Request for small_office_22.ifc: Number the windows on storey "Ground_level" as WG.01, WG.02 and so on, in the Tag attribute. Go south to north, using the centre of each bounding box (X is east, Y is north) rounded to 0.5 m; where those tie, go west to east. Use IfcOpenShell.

First a look at what the model holds.

```python
import ifcopenshell
import ifcopenshell.util.element
import ifcopenshell.util.placement

model = ifcopenshell.open("small_office_22.ifc")
print(model.schema)
storey = next(s for s in model.by_type("IfcBuildingStorey") if s.Name == "Ground_level")
windows = [e for e in ifcopenshell.util.element.get_decomposition(storey) if e.is_a("IfcWindow")]
for e in sorted(windows, key=lambda e: e.id()):
    origin = ifcopenshell.util.placement.get_local_placement(e.ObjectPlacement)[:3, 3]
    print(e.id(), e.Tag, e.Name, origin.round(2) + 0.0, sep=" | ")
```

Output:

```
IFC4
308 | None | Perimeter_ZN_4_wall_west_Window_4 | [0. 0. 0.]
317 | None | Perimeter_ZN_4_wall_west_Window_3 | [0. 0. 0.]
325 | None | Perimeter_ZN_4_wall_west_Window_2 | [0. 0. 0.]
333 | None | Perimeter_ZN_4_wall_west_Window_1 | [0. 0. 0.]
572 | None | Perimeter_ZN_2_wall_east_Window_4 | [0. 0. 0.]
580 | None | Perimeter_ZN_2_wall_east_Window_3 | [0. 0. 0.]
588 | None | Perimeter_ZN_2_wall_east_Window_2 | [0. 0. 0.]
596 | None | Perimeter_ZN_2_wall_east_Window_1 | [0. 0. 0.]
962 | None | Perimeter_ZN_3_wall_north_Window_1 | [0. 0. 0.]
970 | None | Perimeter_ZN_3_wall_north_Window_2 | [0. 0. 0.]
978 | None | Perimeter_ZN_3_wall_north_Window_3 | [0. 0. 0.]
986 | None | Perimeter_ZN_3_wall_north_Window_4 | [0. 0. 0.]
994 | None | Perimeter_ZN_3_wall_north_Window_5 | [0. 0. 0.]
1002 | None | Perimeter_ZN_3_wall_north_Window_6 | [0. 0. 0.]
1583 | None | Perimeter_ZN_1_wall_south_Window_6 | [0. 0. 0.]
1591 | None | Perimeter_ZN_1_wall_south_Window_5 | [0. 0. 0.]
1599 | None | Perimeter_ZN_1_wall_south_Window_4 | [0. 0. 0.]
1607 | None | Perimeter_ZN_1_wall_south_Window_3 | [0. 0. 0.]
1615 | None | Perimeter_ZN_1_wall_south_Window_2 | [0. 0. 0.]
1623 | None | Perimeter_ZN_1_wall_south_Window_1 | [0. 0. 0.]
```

```python
import ifcopenshell
import ifcopenshell.geom
import ifcopenshell.util.element
import ifcopenshell.util.shape

model = ifcopenshell.open("small_office_22.ifc")
settings = ifcopenshell.geom.settings()
settings.set("use-world-coords", True)


def centre(element):
    shape = ifcopenshell.geom.create_shape(settings, element)
    return ifcopenshell.util.shape.get_bbox_centroid(shape.geometry)


storey = next(s for s in model.by_type("IfcBuildingStorey") if s.Name == "Ground_level")
windows = [e for e in ifcopenshell.util.element.get_decomposition(storey) if e.is_a("IfcWindow")]

# Insertion points can sit at a corner or the storey origin, so sort by the geometry (in metres).
centres = {e: centre(e) for e in windows}
windows.sort(key=lambda e: (round(centres[e][1] / 0.5), centres[e][0]))

for i, e in enumerate(windows, start=1):
    number = f"WG.{i:02d}"
    e.Tag = number
    print(e.id(), number)

model.write("small_office_22_rev.ifc")
```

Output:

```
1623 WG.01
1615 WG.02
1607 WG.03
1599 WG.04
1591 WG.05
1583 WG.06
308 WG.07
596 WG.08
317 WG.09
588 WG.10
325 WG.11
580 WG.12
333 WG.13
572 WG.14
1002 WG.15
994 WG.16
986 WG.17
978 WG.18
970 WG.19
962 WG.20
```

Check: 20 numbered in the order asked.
